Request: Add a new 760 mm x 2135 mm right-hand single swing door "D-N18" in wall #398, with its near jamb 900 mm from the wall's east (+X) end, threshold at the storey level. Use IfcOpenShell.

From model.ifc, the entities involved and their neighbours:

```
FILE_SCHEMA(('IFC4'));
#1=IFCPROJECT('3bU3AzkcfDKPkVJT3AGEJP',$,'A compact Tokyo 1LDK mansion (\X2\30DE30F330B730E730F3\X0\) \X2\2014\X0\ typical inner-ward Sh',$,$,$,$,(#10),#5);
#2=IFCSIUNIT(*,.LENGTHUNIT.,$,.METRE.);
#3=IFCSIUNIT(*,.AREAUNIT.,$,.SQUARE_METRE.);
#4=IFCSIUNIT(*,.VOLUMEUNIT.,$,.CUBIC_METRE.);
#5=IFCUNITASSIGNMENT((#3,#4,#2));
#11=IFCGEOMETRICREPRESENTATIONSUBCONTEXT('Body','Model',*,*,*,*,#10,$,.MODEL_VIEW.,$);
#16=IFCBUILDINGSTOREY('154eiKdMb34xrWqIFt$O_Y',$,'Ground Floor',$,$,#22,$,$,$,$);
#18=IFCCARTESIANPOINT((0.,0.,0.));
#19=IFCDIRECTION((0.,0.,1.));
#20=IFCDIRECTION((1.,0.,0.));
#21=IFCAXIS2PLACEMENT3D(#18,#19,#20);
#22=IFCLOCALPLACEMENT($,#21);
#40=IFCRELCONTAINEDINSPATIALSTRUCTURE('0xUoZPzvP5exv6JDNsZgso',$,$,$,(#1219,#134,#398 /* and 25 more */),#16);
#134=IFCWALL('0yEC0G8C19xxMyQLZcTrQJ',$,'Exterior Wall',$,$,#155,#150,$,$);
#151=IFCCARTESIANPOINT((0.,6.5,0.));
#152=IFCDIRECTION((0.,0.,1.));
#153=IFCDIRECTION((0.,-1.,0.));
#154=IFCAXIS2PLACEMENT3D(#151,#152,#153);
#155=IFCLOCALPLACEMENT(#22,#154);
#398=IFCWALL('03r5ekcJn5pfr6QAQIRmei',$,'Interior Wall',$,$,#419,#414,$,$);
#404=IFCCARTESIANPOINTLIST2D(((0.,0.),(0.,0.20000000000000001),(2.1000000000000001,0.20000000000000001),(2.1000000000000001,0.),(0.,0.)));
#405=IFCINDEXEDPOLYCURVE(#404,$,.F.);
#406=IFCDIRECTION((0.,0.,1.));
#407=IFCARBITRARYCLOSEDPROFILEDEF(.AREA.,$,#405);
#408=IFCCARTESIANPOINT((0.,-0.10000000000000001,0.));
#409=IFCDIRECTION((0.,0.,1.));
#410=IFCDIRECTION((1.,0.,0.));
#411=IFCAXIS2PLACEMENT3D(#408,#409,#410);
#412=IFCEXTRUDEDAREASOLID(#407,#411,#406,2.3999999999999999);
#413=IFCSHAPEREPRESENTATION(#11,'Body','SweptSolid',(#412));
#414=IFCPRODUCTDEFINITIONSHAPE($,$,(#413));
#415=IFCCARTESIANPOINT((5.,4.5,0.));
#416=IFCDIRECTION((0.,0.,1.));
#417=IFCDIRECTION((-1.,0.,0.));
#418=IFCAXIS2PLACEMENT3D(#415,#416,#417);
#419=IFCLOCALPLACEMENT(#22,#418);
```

```python
import numpy as np
import ifcopenshell
import ifcopenshell.api.feature
import ifcopenshell.api.geometry
import ifcopenshell.api.root
import ifcopenshell.api.spatial
import ifcopenshell.geom
import ifcopenshell.util.element
import ifcopenshell.util.placement
import ifcopenshell.util.representation
import ifcopenshell.util.shape
import ifcopenshell.util.unit

model = ifcopenshell.open("model.ifc")
unit_scale = ifcopenshell.util.unit.calculate_unit_scale(model)
settings = ifcopenshell.geom.settings()


def volume(element):
    """Net volume in cubic metres, openings subtracted."""
    shape = ifcopenshell.geom.create_shape(settings, element)
    return ifcopenshell.util.shape.get_volume(shape.geometry)


wall = model.by_guid("03r5ekcJn5pfr6QAQIRmei")
storey = ifcopenshell.util.element.get_container(wall, ifc_class="IfcBuildingStorey")
context = ifcopenshell.util.representation.get_context(model, "Model", "Body", "MODEL_VIEW")
before = volume(wall)

width, height, from_end, sill = 0.76, 2.135, 0.9, 0.0  # metres

# The wall runs along its own X axis, and the end named is its -X end.
wall_shape = ifcopenshell.geom.create_shape(settings, wall)
x, y, z = ifcopenshell.util.shape.get_vertices(wall_shape.geometry).T
start = x.min() + from_end
face, thickness = float(y.min()), float(y.max() - y.min())
wall_matrix = ifcopenshell.util.placement.get_local_placement(wall.ObjectPlacement)
level = ifcopenshell.util.placement.get_local_placement(storey.ObjectPlacement)[2, 3]


def in_wall(x, y):
    """Placement at x, y metres in the wall's axes, at sill height."""
    matrix = wall_matrix.copy()
    matrix[:, 3] = wall_matrix @ np.array([x / unit_scale, y / unit_scale, 0.0, 1.0])
    matrix[2, 3] = level + sill / unit_scale
    return matrix


# Opening: a box that overshoots both wall faces by 50 mm.
opening = ifcopenshell.api.root.create_entity(model, ifc_class="IfcOpeningElement", predefined_type="OPENING")
box = ifcopenshell.api.geometry.add_wall_representation(
    model, context=context, length=width, height=height, thickness=thickness + 0.1
)
ifcopenshell.api.geometry.assign_representation(model, product=opening, representation=box)
ifcopenshell.api.geometry.edit_object_placement(model, product=opening, matrix=in_wall(start, face - 0.05), is_si=False)
ifcopenshell.api.feature.add_feature(model, feature=opening, element=wall)

door = ifcopenshell.api.root.create_entity(model, ifc_class="IfcDoor", name="D-N18", predefined_type="DOOR")
door.OverallWidth, door.OverallHeight = width / unit_scale, height / unit_scale
door.OperationType = "SINGLE_SWING_RIGHT"
body = ifcopenshell.api.geometry.add_door_representation(
    model,
    context=context,
    overall_width=door.OverallWidth,
    overall_height=door.OverallHeight,
    operation_type="SINGLE_SWING_RIGHT",
    lining_properties={"LiningDepth": thickness / unit_scale, "ThresholdDepth": thickness / unit_scale},
)
ifcopenshell.api.geometry.assign_representation(model, product=door, representation=body)
ifcopenshell.api.spatial.assign_container(model, products=[door], relating_structure=storey)
ifcopenshell.api.feature.add_filling(model, opening=opening, element=door)

# The lining spans the wall, so the door starts at the wall face.
ifcopenshell.api.geometry.edit_object_placement(model, product=door, matrix=in_wall(start, face), is_si=False)

after = volume(wall)

print(f"wall volume {before:.3f} -> {after:.3f} m3")

model.write("model_v2.ifc")
```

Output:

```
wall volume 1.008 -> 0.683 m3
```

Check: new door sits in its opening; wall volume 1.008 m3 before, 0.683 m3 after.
